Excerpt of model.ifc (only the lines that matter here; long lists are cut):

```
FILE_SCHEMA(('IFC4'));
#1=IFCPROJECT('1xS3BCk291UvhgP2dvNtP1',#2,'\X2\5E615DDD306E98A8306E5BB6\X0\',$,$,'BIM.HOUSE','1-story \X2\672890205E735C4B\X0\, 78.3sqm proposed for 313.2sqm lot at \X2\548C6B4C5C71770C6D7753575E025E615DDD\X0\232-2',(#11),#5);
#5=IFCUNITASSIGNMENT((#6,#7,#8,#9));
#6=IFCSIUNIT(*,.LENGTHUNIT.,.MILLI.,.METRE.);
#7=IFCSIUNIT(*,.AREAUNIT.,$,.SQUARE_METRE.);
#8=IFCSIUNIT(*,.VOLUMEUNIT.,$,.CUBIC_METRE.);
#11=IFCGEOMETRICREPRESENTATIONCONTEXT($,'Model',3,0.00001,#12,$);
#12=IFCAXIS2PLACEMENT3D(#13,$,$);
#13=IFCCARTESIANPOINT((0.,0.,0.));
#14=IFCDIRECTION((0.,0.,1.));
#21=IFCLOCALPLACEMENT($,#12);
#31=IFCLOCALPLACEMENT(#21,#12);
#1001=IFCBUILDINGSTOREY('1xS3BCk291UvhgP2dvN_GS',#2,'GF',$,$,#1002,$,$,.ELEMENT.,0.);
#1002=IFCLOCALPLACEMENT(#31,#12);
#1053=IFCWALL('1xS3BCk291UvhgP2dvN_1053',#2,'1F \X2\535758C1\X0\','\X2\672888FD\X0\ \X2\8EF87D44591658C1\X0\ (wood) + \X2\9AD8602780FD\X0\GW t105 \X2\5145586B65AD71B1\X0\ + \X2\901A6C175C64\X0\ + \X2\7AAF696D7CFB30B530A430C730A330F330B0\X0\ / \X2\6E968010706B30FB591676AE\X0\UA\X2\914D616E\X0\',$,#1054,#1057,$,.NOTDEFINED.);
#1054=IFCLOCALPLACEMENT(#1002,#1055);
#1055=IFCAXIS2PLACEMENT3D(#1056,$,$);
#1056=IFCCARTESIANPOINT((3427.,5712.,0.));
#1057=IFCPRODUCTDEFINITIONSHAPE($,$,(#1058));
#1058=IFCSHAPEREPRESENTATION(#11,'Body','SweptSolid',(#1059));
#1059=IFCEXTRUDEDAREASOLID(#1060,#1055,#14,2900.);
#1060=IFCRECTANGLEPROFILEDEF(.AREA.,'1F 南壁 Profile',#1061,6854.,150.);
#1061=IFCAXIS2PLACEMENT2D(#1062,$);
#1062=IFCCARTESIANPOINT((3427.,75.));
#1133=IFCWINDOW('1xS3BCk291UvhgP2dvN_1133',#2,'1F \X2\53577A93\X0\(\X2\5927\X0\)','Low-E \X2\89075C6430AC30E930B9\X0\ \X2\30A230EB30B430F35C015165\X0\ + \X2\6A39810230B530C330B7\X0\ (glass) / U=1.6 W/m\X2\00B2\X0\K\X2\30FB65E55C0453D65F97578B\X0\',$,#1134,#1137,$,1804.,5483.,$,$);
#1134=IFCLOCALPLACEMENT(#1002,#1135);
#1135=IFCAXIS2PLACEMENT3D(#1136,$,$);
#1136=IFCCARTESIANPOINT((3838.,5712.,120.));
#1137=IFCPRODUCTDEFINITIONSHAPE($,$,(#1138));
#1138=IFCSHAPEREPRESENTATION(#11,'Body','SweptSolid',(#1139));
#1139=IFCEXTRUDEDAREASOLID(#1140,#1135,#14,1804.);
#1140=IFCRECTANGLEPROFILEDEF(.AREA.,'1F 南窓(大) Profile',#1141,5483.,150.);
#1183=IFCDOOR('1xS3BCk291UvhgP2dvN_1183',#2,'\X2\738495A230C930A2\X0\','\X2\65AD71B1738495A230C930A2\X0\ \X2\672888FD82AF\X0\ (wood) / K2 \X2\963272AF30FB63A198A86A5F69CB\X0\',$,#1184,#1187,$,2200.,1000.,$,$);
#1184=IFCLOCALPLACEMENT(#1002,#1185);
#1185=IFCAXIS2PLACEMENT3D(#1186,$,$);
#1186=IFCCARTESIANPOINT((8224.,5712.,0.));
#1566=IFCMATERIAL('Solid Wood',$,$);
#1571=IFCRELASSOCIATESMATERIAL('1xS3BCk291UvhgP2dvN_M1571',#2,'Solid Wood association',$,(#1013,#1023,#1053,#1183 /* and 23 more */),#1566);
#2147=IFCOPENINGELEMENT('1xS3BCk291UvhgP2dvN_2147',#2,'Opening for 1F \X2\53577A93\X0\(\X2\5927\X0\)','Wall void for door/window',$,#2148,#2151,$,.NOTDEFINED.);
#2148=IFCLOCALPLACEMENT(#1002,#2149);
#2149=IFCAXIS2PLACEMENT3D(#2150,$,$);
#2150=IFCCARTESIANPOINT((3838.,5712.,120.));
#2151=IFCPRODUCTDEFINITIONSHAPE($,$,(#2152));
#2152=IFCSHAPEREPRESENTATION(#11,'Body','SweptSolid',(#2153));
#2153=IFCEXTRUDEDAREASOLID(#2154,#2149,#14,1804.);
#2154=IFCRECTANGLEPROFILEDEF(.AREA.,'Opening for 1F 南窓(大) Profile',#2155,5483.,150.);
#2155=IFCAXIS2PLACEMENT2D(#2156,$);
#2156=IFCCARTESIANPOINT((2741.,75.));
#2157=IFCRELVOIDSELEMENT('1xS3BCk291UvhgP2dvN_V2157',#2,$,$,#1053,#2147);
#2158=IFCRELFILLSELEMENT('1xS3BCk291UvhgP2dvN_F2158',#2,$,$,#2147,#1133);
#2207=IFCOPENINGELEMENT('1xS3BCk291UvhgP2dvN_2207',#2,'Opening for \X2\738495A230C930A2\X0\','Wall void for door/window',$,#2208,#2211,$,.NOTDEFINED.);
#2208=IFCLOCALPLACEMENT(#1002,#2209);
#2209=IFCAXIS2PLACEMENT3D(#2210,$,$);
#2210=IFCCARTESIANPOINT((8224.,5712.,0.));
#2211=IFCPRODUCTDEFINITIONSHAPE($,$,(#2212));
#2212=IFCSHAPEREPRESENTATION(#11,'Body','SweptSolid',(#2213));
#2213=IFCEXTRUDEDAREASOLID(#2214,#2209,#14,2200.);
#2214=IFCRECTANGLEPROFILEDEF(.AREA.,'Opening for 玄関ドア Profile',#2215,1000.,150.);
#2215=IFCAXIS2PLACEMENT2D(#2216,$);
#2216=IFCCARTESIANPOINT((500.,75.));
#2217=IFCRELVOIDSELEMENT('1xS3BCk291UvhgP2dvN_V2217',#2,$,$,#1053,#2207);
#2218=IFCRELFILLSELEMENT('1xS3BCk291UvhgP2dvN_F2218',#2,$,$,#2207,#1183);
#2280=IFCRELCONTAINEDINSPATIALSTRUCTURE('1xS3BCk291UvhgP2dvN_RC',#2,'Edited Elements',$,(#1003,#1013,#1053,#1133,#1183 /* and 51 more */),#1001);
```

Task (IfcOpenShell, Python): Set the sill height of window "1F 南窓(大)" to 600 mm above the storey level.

```python
import numpy as np
import ifcopenshell
import ifcopenshell.api.geometry
import ifcopenshell.geom
import ifcopenshell.util.element
import ifcopenshell.util.placement
import ifcopenshell.util.shape
import ifcopenshell.util.unit

model = ifcopenshell.open("model.ifc")
unit_scale = ifcopenshell.util.unit.calculate_unit_scale(model)

window = model.by_guid("1xS3BCk291UvhgP2dvN_1133")
opening = window.FillsVoids[0].RelatingOpeningElement
storey = ifcopenshell.util.element.get_container(window, ifc_class="IfcBuildingStorey")
level = ifcopenshell.util.placement.get_local_placement(storey.ObjectPlacement)[2, 3]

# The opening's origin need not be at the sill, so measure its lowest point.
shape = ifcopenshell.geom.create_shape(ifcopenshell.geom.settings(), opening)
bottom = ifcopenshell.util.shape.get_shape_bottom_elevation(shape, shape.geometry) / unit_scale
dz = level + 0.6 / unit_scale - bottom

shift = np.array([0.0, 0.0, dz])
# The window is not placed relative to its opening, so move both.
for product in (opening, window):
    matrix = ifcopenshell.util.placement.get_local_placement(product.ObjectPlacement)
    matrix[:3, 3] += shift
    ifcopenshell.api.geometry.edit_object_placement(model, product=product, matrix=matrix, is_si=False)

print(f"moved by {dz * unit_scale:+.3f} m")

model.write("model_updated.ifc")
```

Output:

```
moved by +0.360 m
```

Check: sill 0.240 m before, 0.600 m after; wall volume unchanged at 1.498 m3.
